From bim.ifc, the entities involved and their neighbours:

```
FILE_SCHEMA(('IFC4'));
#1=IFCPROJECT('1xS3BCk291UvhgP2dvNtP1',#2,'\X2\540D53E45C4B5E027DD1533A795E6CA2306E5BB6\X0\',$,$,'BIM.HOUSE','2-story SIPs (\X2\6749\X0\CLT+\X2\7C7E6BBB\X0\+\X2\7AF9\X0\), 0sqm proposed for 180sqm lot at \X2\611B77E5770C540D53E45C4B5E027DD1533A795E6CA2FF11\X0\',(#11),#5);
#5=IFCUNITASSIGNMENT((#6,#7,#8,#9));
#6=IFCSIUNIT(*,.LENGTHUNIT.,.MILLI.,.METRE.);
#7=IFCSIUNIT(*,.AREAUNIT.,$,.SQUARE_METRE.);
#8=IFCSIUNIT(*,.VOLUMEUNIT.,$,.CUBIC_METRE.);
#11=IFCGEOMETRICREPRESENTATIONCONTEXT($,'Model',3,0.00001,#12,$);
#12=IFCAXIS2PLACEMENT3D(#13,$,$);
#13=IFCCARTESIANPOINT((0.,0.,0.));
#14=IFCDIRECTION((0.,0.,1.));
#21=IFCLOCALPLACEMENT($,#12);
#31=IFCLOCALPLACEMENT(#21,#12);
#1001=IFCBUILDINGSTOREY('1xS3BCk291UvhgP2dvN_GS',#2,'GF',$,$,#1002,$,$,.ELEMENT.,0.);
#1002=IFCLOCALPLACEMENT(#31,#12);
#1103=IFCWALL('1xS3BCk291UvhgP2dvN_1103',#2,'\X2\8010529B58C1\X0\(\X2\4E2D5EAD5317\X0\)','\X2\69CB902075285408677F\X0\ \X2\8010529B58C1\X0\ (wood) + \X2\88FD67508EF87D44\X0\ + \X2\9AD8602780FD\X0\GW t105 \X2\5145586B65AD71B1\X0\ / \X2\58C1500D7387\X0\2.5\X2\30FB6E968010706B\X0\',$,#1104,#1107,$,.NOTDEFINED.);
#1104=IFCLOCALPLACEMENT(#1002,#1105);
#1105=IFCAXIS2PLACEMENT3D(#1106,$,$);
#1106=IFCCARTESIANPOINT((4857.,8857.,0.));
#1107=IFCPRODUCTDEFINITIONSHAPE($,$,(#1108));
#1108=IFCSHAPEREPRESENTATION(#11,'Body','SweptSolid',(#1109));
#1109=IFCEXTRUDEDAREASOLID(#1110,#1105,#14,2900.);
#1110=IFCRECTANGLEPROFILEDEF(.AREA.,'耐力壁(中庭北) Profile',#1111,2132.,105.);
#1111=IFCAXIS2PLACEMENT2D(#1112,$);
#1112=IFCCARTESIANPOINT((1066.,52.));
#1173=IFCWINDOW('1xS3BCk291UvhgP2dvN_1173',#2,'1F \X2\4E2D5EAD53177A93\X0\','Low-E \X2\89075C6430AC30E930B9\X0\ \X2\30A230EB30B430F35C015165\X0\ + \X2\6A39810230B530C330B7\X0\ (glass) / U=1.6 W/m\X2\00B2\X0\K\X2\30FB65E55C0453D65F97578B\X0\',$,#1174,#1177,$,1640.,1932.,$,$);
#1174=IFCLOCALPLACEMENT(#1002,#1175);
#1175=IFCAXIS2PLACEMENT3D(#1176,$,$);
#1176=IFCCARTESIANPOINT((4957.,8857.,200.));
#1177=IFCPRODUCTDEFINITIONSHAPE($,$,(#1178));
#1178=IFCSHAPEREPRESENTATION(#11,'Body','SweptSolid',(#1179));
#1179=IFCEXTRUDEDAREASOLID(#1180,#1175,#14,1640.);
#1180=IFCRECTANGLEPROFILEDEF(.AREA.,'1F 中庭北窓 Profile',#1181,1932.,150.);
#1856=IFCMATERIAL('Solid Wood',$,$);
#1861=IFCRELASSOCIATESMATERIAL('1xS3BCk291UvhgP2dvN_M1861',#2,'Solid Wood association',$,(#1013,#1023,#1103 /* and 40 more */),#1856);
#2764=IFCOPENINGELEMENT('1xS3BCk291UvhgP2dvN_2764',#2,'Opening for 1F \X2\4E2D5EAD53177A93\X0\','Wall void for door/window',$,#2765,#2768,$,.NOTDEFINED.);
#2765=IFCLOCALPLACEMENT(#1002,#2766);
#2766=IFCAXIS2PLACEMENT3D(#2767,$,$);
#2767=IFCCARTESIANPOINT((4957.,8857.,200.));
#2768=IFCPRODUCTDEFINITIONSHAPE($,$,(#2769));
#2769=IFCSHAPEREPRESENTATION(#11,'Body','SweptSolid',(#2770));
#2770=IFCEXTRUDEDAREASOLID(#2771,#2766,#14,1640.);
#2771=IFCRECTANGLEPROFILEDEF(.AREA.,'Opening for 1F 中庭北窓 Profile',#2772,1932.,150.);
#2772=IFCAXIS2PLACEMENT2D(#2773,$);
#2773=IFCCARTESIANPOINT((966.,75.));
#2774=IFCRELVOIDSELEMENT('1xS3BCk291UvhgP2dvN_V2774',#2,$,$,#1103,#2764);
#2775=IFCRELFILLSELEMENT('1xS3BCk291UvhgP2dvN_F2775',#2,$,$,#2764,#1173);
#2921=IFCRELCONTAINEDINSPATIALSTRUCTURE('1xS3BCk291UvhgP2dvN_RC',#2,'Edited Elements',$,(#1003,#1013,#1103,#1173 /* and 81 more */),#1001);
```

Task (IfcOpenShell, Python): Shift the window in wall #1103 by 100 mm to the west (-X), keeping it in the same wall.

```python
import ifcopenshell
import ifcopenshell.api.geometry
import ifcopenshell.util.placement
import ifcopenshell.util.unit

model = ifcopenshell.open("bim.ifc")
unit_scale = ifcopenshell.util.unit.calculate_unit_scale(model)

window = model.by_guid("1xS3BCk291UvhgP2dvN_1173")
opening = window.FillsVoids[0].RelatingOpeningElement
wall = opening.VoidsElements[0].RelatingBuildingElement

wall_matrix = ifcopenshell.util.placement.get_local_placement(wall.ObjectPlacement)
shift = wall_matrix[:3, 0] * -0.1 / unit_scale
before = ifcopenshell.util.placement.get_local_placement(window.ObjectPlacement)[:3, 3].copy()

# The window is not placed relative to its opening, so move both.
for product in (opening, window):
    matrix = ifcopenshell.util.placement.get_local_placement(product.ObjectPlacement)
    matrix[:3, 3] += shift
    ifcopenshell.api.geometry.edit_object_placement(model, product=product, matrix=matrix, is_si=False)

after = ifcopenshell.util.placement.get_local_placement(window.ObjectPlacement)[:3, 3]
print("window moved by", (after - before).round(3) + 0.0)

model.write("bim_updated.ifc")
```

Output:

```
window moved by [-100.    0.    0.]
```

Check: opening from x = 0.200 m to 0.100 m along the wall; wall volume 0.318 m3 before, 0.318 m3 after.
